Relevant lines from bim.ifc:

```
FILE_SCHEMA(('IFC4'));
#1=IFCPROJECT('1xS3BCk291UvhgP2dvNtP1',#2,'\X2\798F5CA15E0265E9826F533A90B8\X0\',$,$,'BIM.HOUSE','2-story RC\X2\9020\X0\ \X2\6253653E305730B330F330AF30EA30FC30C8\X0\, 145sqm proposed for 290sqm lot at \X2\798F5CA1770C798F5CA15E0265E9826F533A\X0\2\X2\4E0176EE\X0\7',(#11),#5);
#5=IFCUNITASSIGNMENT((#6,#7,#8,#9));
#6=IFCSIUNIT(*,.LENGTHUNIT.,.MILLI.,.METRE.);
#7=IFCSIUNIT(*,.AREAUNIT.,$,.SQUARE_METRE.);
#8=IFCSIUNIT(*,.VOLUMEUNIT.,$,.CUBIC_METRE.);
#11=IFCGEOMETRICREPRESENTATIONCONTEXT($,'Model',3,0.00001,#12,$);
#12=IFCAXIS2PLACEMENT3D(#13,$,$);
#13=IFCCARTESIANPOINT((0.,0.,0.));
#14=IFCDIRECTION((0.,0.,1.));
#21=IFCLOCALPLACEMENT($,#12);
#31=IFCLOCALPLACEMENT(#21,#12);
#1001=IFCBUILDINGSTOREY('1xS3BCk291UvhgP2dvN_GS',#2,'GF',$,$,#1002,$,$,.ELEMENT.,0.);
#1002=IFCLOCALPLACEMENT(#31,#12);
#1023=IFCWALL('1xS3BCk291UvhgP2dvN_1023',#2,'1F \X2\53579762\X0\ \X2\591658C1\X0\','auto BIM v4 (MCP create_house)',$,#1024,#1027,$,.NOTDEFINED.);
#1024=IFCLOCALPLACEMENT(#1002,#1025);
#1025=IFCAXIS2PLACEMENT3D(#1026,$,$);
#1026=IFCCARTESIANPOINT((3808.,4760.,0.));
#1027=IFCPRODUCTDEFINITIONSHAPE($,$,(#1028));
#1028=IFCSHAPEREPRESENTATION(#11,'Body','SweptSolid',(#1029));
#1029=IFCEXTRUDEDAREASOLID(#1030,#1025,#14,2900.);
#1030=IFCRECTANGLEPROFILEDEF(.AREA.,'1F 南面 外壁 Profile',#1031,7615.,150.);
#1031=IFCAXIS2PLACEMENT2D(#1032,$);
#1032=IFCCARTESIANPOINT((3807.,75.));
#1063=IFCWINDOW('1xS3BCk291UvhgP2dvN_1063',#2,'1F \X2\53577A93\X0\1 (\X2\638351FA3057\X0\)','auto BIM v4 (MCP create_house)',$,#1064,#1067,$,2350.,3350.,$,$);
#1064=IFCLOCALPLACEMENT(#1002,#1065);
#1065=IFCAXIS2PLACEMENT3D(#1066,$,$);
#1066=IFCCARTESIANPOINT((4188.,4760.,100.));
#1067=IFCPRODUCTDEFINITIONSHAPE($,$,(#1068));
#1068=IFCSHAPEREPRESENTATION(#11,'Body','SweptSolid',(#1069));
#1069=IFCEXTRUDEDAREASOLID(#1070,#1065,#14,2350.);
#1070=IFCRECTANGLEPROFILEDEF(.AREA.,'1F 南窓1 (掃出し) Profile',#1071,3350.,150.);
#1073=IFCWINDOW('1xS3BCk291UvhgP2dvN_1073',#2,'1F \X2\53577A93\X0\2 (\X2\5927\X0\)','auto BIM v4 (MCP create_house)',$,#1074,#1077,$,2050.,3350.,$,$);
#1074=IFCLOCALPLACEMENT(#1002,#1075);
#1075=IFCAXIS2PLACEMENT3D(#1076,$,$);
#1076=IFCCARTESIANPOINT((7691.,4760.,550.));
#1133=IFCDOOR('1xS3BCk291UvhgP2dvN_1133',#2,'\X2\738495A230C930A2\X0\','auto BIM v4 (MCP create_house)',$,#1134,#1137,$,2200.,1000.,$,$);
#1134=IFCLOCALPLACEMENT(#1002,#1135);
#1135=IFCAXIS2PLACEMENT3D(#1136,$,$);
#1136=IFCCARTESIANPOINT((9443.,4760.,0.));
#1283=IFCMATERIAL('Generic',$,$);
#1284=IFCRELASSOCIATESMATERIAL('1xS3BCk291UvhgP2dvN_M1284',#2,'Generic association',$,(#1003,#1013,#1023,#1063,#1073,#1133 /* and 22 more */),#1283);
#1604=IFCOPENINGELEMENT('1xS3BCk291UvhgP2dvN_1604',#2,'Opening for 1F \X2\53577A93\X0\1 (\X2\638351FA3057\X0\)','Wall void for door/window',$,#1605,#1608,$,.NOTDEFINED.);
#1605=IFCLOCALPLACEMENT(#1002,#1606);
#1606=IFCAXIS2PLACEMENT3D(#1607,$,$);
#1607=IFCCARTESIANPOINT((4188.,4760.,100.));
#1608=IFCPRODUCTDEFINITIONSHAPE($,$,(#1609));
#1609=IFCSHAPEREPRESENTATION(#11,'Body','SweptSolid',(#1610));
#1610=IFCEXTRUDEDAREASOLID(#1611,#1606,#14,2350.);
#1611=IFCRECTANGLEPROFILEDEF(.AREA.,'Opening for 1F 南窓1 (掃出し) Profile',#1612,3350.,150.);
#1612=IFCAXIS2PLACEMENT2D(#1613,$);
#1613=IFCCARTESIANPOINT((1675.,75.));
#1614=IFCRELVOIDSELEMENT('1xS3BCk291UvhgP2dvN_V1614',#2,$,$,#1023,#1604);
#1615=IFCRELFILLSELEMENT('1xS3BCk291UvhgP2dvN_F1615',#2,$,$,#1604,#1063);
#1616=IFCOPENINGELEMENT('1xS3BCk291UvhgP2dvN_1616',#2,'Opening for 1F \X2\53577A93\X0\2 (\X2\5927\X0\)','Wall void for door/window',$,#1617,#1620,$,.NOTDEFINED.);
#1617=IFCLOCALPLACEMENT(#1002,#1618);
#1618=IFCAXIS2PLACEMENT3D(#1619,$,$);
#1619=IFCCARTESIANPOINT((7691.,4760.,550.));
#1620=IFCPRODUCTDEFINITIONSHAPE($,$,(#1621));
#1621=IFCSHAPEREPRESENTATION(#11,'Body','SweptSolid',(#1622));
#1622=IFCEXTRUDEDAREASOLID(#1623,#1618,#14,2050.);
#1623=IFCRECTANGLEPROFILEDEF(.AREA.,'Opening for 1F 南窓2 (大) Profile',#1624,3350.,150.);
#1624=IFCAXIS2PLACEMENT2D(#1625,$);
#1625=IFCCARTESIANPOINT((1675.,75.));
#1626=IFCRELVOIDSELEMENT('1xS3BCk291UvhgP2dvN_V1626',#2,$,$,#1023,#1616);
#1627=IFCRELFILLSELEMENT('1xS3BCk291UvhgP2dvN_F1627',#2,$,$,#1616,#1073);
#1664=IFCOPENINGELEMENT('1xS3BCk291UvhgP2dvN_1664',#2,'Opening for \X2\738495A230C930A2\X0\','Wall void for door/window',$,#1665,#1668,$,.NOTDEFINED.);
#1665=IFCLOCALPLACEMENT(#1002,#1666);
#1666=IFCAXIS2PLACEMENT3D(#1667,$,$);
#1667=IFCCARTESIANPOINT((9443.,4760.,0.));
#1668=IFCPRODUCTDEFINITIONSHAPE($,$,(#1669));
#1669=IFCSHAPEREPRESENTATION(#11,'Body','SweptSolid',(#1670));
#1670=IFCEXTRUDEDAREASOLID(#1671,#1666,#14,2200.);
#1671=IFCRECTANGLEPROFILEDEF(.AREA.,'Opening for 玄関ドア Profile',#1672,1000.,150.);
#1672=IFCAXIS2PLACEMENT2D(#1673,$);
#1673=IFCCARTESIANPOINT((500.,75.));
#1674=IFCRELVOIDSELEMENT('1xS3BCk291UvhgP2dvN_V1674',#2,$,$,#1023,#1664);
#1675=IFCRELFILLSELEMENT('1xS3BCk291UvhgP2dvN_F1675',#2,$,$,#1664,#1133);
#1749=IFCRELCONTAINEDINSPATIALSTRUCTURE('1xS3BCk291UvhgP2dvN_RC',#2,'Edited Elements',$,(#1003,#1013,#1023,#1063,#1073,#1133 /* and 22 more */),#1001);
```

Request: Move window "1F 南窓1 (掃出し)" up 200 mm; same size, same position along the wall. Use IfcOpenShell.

```python
import numpy as np
import ifcopenshell
import ifcopenshell.api.geometry
import ifcopenshell.util.placement
import ifcopenshell.util.unit

model = ifcopenshell.open("bim.ifc")
unit_scale = ifcopenshell.util.unit.calculate_unit_scale(model)

window = model.by_guid("1xS3BCk291UvhgP2dvN_1063")
opening = window.FillsVoids[0].RelatingOpeningElement
dz = 0.2 / unit_scale

shift = np.array([0.0, 0.0, dz])
# The window is not placed relative to its opening, so move both.
for product in (opening, window):
    matrix = ifcopenshell.util.placement.get_local_placement(product.ObjectPlacement)
    matrix[:3, 3] += shift
    ifcopenshell.api.geometry.edit_object_placement(model, product=product, matrix=matrix, is_si=False)

print(f"moved by {dz * unit_scale:+.3f} m")

model.write("bim_edited.ifc")
```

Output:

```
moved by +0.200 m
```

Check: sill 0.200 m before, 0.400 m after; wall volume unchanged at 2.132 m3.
